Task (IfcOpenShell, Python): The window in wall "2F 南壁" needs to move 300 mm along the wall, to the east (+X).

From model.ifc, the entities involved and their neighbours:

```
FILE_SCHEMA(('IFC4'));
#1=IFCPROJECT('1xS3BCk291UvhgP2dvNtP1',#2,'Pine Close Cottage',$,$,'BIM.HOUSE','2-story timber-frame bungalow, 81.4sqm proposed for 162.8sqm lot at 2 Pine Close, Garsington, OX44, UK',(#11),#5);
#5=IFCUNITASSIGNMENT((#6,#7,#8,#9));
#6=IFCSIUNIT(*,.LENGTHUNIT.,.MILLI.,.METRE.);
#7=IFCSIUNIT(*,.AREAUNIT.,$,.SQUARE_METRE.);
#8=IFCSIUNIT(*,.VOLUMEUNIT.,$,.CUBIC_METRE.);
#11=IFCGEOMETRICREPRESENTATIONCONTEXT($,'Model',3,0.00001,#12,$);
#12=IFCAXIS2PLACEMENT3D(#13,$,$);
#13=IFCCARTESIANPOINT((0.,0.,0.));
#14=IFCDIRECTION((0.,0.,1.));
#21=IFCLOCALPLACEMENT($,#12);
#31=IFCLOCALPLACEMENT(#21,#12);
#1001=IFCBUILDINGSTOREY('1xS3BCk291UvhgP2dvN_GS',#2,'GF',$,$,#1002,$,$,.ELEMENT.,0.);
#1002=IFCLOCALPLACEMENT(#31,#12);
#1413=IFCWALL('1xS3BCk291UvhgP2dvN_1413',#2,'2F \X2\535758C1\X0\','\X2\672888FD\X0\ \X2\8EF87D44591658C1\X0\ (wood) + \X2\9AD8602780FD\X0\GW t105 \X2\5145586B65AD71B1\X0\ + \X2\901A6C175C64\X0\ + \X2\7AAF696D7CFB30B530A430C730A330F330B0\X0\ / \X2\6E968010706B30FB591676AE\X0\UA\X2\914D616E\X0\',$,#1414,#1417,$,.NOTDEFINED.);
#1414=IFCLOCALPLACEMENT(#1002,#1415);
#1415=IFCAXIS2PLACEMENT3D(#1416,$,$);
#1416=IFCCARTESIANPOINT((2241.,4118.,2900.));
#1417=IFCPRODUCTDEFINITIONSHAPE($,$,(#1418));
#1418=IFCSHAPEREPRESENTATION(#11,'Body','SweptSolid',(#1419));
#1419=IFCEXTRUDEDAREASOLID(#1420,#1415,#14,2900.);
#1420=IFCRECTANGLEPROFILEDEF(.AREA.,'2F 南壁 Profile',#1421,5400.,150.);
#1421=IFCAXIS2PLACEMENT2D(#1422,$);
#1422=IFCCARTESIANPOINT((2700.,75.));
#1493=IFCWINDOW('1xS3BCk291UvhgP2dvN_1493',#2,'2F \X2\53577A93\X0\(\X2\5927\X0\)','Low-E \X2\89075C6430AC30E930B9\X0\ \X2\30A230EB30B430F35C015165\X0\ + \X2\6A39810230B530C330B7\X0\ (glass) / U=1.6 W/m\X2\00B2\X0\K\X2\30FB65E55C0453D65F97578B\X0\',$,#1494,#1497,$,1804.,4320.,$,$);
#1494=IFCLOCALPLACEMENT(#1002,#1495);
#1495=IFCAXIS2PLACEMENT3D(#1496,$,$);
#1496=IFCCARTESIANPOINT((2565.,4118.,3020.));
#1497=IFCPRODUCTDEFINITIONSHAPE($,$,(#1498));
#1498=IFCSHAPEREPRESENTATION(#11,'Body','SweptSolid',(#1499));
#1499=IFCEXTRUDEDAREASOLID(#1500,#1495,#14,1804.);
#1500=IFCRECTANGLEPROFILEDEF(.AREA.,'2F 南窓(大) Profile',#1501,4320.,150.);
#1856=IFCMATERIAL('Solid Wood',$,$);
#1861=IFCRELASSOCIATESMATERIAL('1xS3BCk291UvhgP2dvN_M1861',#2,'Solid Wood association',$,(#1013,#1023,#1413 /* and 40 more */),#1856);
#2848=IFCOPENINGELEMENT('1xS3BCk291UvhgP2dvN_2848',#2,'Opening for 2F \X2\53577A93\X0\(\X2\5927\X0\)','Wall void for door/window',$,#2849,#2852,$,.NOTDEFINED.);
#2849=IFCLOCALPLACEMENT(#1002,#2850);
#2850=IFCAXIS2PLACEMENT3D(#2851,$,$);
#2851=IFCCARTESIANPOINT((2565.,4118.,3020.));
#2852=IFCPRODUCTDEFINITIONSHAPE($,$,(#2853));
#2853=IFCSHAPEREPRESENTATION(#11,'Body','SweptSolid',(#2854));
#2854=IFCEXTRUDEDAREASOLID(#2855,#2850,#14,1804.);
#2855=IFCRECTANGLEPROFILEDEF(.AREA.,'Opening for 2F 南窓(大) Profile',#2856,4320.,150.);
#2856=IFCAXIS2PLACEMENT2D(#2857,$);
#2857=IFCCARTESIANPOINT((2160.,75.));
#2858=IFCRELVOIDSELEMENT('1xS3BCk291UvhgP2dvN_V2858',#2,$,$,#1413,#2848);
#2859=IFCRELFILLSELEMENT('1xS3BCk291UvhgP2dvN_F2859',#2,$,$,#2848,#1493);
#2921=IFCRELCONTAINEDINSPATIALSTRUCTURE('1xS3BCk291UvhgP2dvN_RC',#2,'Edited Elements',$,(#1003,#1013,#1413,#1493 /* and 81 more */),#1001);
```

```python
import ifcopenshell
import ifcopenshell.api.geometry
import ifcopenshell.util.placement

model = ifcopenshell.open("model.ifc")

window = model.by_guid("1xS3BCk291UvhgP2dvN_1493")
opening = window.FillsVoids[0].RelatingOpeningElement
wall = opening.VoidsElements[0].RelatingBuildingElement

wall_matrix = ifcopenshell.util.placement.get_local_placement(wall.ObjectPlacement)
shift = wall_matrix[:3, 0] * 300.0
before = ifcopenshell.util.placement.get_local_placement(window.ObjectPlacement)[:3, 3].copy()

# The window is not placed relative to its opening, so move both.
for product in (opening, window):
    matrix = ifcopenshell.util.placement.get_local_placement(product.ObjectPlacement)
    matrix[:3, 3] += shift
    ifcopenshell.api.geometry.edit_object_placement(model, product=product, matrix=matrix, is_si=False)

after = ifcopenshell.util.placement.get_local_placement(window.ObjectPlacement)[:3, 3]
print("window moved by", (after - before).round(3) + 0.0)

model.write("model-out.ifc")
```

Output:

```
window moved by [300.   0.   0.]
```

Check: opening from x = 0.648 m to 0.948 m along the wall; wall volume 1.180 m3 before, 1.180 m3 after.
